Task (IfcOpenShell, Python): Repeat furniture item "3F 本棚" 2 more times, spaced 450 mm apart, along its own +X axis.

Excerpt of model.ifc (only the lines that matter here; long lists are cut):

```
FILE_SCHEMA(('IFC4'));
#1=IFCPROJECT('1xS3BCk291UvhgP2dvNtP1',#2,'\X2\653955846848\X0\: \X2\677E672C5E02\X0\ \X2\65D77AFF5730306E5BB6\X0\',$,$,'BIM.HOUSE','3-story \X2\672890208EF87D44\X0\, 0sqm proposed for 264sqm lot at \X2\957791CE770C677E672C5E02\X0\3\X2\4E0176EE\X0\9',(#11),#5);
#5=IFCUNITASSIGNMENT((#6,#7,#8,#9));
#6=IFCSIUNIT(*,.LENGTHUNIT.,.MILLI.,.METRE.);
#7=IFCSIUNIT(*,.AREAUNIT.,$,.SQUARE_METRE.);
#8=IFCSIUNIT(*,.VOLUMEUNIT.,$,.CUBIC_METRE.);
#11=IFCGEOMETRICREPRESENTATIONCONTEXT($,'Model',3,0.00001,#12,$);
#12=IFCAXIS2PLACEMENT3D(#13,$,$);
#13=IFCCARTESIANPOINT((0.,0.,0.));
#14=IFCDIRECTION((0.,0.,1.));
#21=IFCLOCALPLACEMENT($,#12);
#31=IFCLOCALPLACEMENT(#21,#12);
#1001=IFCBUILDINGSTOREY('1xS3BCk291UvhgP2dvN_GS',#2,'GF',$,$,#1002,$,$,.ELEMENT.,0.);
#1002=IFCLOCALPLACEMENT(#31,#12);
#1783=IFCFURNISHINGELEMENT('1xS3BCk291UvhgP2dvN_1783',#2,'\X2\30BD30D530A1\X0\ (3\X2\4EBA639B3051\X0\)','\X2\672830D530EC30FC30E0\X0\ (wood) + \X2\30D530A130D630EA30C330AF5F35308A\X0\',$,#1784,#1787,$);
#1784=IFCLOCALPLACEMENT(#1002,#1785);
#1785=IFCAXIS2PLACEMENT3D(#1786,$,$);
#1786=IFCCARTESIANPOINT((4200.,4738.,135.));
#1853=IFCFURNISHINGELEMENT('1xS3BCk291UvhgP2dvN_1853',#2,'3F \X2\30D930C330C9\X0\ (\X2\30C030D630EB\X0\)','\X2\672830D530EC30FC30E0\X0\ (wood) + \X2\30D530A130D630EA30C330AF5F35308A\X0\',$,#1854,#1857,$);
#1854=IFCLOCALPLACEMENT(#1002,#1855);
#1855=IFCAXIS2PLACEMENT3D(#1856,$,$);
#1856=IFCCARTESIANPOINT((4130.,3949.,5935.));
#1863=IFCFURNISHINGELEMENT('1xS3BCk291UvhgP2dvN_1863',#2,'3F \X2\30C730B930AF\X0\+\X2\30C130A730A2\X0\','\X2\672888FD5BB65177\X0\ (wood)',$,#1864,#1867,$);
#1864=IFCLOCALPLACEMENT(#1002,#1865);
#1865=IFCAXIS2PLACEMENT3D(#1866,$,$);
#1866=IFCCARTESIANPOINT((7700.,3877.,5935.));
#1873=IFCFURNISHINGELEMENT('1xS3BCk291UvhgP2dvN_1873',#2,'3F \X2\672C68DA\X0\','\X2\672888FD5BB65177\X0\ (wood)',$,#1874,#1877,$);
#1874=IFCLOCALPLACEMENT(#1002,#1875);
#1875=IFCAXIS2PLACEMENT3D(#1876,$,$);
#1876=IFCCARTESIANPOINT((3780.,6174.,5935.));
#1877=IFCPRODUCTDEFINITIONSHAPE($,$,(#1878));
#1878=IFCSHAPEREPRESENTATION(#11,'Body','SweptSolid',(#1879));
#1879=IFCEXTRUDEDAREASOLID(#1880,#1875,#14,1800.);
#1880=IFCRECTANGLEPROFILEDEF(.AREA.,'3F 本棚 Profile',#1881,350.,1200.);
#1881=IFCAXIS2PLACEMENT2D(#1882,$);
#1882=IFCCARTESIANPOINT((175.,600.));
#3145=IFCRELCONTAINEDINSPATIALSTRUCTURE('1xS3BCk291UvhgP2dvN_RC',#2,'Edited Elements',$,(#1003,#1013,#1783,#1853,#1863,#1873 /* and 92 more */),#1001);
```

```python
import ifcopenshell
import ifcopenshell.api.geometry
import ifcopenshell.api.root
import ifcopenshell.util.element
import ifcopenshell.util.placement
import ifcopenshell.util.unit

model = ifcopenshell.open("model.ifc")
unit_scale = ifcopenshell.util.unit.calculate_unit_scale(model)


def reuse_history(source, copy):
    """copy_class also copies each property set's owner history, people and application; keep the originals."""
    for rel in copy.IsDefinedBy:
        if rel.is_a("IfcRelDefinesByProperties") and (history := rel.RelatingPropertyDefinition.OwnerHistory):
            rel.RelatingPropertyDefinition.OwnerHistory = source.OwnerHistory
            ifcopenshell.util.element.remove_deep2(model, history)


source = model.by_guid("1xS3BCk291UvhgP2dvN_1873")
base = ifcopenshell.util.placement.get_local_placement(source.ObjectPlacement)
step = base[:3, 0] * 0.45 / unit_scale

for i in range(1, 3):
    copy = ifcopenshell.api.root.copy_class(model, product=source)
    copy.Representation = ifcopenshell.util.element.copy_deep(
        model, source.Representation, exclude=["IfcGeometricRepresentationContext", "IfcRepresentationMap"]
    )
    reuse_history(source, copy)
    matrix = base.copy()
    matrix[:3, 3] += i * step
    print("added at", matrix[:3, 3].round(3) + 0.0)
    ifcopenshell.api.geometry.edit_object_placement(model, product=copy, matrix=matrix, is_si=False)

model.write("model_rev.ifc")
```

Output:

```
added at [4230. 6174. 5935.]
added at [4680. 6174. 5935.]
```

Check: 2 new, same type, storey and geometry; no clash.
